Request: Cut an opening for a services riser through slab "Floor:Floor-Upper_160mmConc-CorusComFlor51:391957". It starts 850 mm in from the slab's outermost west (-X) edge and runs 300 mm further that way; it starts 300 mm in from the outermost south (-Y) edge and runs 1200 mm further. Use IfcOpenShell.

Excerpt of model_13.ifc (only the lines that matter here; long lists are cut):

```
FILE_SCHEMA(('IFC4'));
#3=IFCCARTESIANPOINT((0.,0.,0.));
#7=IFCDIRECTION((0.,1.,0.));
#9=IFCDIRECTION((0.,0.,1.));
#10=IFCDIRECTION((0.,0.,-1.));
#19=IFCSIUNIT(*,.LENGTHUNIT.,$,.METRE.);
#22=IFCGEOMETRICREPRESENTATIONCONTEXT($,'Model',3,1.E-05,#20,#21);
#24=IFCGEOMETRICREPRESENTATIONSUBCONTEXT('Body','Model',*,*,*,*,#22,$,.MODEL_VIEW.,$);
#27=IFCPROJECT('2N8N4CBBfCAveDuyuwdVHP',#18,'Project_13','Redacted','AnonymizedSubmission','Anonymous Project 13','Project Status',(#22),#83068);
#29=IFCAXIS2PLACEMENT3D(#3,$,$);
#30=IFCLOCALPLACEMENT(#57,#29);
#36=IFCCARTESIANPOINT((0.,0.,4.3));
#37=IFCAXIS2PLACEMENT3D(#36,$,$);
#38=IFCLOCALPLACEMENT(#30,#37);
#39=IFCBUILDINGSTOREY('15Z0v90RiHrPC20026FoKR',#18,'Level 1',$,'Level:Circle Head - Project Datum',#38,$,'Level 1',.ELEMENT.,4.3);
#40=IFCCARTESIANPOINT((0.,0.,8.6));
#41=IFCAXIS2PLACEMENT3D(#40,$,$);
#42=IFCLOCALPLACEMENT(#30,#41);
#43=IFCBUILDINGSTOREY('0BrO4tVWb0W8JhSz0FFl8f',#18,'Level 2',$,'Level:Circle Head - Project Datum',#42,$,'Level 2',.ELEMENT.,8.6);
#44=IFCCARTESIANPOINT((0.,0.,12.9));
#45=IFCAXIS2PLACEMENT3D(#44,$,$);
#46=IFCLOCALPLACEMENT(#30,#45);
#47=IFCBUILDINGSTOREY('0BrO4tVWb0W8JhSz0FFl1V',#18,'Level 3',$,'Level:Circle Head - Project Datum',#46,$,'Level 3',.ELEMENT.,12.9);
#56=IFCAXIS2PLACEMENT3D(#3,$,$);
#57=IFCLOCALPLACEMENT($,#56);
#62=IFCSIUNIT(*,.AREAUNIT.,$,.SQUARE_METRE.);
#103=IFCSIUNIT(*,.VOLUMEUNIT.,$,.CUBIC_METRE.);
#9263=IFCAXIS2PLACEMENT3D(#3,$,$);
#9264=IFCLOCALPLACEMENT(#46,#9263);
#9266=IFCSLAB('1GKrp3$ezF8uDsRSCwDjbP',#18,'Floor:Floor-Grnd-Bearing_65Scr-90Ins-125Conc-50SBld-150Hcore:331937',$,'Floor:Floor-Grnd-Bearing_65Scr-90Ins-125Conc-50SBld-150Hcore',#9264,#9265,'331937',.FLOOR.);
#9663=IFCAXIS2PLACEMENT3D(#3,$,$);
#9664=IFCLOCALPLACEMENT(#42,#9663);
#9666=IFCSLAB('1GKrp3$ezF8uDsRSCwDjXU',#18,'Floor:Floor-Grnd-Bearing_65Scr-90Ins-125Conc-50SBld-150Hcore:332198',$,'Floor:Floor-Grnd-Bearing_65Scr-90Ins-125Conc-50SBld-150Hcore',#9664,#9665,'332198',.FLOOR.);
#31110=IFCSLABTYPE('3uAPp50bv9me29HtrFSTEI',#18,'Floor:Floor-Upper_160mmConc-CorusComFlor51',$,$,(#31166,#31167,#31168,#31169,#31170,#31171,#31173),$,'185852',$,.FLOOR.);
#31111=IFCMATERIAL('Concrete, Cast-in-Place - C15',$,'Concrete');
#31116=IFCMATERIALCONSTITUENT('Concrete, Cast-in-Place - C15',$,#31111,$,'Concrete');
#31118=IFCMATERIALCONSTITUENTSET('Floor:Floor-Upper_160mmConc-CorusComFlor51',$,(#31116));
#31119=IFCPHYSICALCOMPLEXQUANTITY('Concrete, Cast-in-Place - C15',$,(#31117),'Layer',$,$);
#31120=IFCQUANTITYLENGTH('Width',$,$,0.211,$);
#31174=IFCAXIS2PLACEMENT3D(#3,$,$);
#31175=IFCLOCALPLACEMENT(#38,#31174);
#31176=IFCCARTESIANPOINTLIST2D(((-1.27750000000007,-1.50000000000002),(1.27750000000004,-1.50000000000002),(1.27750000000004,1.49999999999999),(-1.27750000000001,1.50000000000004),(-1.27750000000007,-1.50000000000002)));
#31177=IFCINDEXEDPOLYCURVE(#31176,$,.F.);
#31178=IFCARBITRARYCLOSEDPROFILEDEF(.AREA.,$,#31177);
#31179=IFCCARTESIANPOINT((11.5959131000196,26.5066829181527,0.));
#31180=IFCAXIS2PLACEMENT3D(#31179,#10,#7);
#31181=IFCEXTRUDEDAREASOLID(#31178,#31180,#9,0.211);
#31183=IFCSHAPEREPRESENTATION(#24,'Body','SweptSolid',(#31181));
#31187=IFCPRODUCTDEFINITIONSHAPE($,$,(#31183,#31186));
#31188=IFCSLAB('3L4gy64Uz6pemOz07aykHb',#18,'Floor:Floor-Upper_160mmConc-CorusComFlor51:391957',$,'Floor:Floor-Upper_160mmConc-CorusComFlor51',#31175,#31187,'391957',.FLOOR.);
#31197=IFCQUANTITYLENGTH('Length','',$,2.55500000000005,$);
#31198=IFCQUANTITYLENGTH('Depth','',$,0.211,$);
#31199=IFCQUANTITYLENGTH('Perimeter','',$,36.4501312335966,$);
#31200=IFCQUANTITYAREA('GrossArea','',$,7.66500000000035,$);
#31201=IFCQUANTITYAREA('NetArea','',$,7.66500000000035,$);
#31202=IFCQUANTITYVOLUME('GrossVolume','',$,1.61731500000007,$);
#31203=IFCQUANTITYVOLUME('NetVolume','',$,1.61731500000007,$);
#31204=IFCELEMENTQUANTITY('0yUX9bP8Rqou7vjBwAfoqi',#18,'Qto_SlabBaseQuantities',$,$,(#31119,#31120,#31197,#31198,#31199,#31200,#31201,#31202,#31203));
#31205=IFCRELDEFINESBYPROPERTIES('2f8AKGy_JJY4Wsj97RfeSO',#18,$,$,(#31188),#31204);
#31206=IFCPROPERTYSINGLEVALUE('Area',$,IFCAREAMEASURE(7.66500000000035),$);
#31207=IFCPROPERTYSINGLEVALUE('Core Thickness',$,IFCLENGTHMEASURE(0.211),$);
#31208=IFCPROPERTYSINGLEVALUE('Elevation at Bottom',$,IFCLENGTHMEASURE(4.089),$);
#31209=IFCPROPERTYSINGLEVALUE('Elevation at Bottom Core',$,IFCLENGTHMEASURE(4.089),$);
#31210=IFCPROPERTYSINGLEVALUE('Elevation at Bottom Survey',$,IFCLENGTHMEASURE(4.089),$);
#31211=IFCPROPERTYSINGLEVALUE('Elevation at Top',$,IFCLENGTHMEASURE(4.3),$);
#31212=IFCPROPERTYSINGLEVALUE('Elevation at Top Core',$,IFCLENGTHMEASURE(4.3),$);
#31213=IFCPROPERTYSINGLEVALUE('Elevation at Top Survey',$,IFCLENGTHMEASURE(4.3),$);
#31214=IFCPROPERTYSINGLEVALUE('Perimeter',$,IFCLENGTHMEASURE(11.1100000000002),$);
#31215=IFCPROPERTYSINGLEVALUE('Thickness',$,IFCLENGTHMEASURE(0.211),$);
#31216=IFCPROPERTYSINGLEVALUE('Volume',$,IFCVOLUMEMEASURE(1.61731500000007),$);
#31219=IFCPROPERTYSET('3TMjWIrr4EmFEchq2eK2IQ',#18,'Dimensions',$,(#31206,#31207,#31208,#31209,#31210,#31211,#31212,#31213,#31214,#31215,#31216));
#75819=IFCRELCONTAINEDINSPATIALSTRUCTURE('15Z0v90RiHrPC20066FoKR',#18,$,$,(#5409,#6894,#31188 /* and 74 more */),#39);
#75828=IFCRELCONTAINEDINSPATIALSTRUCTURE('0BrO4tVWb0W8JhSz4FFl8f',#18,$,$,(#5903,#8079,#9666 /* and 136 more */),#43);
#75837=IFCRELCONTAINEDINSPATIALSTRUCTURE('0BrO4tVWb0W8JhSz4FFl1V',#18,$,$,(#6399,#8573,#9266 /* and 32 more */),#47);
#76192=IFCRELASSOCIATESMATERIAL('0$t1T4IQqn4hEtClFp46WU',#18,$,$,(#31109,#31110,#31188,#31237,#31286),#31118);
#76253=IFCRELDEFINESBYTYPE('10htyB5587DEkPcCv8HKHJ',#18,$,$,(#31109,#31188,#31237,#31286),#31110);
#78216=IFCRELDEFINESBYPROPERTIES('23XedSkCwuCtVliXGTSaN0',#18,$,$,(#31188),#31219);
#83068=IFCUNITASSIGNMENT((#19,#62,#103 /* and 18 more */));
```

```python
import numpy as np
import ifcopenshell
import ifcopenshell.api.feature
import ifcopenshell.api.geometry
import ifcopenshell.api.pset
import ifcopenshell.api.root
import ifcopenshell.geom
import ifcopenshell.util.element
import ifcopenshell.util.placement
import ifcopenshell.util.representation
import ifcopenshell.util.shape
import ifcopenshell.util.unit

model = ifcopenshell.open("model_13.ifc")
unit_scale = ifcopenshell.util.unit.calculate_unit_scale(model)
area_scale = ifcopenshell.util.unit.calculate_unit_scale(model, "AREAUNIT")
volume_scale = ifcopenshell.util.unit.calculate_unit_scale(model, "VOLUMEUNIT")
settings = ifcopenshell.geom.settings()


def volume(element):
    """Net volume in cubic metres, openings subtracted."""
    shape = ifcopenshell.geom.create_shape(settings, element)
    return ifcopenshell.util.shape.get_volume(shape.geometry)


slab = model.by_guid("3L4gy64Uz6pemOz07aykHb")
before = volume(slab)

# Extent in the slab's own axes, in metres. The edges named are its -X and -Y sides.
slab_shape = ifcopenshell.geom.create_shape(settings, slab)
vertices = ifcopenshell.util.shape.get_vertices(slab_shape.geometry)
x_min, y_min, bottom = vertices.min(axis=0)
top = vertices[:, 2].max()

opening = ifcopenshell.api.root.create_entity(model, ifc_class="IfcOpeningElement", name="Services riser opening", predefined_type="OPENING")
context = ifcopenshell.util.representation.get_context(model, "Model", "Body", "MODEL_VIEW")
width, depth = 0.3, 1.2
outline = [(0.0, 0.0), (width, 0.0), (width, depth), (0.0, depth), (0.0, 0.0)]
# Overshoot both faces by 50 mm so the cut is clean.
shape = ifcopenshell.api.geometry.add_slab_representation(
    model, context=context, depth=top - bottom + 0.1, polyline=outline
)
ifcopenshell.api.geometry.assign_representation(model, product=opening, representation=shape)

matrix = ifcopenshell.util.placement.get_local_placement(slab.ObjectPlacement)
matrix[:, 3] = matrix @ np.append(np.array([x_min + 0.85, y_min + 0.3, bottom - 0.05]) / unit_scale, 1.0)
ifcopenshell.api.geometry.edit_object_placement(model, product=opening, matrix=matrix, is_si=False)
ifcopenshell.api.feature.add_feature(model, feature=opening, element=slab)

after = volume(slab)

# Update the slab's stored quantities.
qto = model.by_id(ifcopenshell.util.element.get_pset(slab, "Qto_SlabBaseQuantities", should_inherit=False)["id"])
ifcopenshell.api.pset.edit_qto(model, qto=qto, properties={
    "NetArea": after / (top - bottom) / area_scale,
    "NetVolume": after / volume_scale,
})
pset = model.by_id(ifcopenshell.util.element.get_pset(slab, "Dimensions", should_inherit=False)["id"])
ifcopenshell.api.pset.edit_pset(model, pset=pset, properties={
    "Area": model.create_entity("IfcAreaMeasure", after / (top - bottom) / area_scale),
    "Volume": model.create_entity("IfcVolumeMeasure", after / volume_scale),
})

print(f"slab volume {before:.3f} -> {after:.3f} m3")

model.write("model_13_rev.ifc")
```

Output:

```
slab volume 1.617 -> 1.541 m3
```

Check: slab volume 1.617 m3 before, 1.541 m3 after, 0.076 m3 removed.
